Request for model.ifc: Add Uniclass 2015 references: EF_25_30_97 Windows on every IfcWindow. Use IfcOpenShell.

First a look at what the model holds.

```python
import ifcopenshell

model = ifcopenshell.open("model.ifc")
print(model.schema)
print("classifications:", [c.Name for c in model.by_type("IfcClassification")])
for ifc_class in ("IfcDoor", "IfcRoof", "IfcStair", "IfcWall", "IfcWindow"):
    print(ifc_class, len(model.by_type(ifc_class)))
```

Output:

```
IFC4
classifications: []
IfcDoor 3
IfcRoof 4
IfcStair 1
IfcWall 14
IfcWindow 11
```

```python
import ifcopenshell
import ifcopenshell.api.classification

model = ifcopenshell.open("model.ifc")

system = ifcopenshell.api.classification.add_classification(model, classification="Uniclass 2015")

codes = {
    "IfcWindow": ("EF_25_30_97", "Windows"),
}
for ifc_class, (code, name) in codes.items():
    products = model.by_type(ifc_class)
    ifcopenshell.api.classification.add_reference(
        model, products=products, classification=system, identification=code, name=name
    )
    print(code, len(products))

model.write("model_v2.ifc")
```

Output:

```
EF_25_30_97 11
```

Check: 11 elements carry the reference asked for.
